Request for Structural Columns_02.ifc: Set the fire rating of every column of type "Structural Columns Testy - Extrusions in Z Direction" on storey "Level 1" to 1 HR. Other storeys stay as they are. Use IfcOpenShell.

First a look at what the model holds.

```python
import ifcopenshell
import ifcopenshell.util.element

model = ifcopenshell.open("Structural Columns_02.ifc")
print(model.schema)
storey = next(s for s in model.by_type("IfcBuildingStorey") if s.Name == "Level 1")
columns = [e for e in ifcopenshell.util.element.get_decomposition(storey) if e.is_a("IfcColumn")]
seen = {}
for e in columns:
    element_type = ifcopenshell.util.element.get_type(e)
    key = (element_type.Name if element_type != e and element_type else None, ifcopenshell.util.element.get_pset(e, "Pset_ColumnCommon", "FireRating"))
    seen[key] = seen.get(key, 0) + 1
for (name, value), count in sorted(seen.items(), key=str):
    print(count, "x", name, "|", value)
```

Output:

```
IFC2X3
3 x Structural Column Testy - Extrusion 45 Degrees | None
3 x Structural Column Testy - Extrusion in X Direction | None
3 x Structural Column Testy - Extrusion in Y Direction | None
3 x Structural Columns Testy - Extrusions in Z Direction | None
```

```python
import ifcopenshell
import ifcopenshell.api.pset
import ifcopenshell.util.element

model = ifcopenshell.open("Structural Columns_02.ifc")

storey = next(s for s in model.by_type("IfcBuildingStorey") if s.Name == "Level 1")
columns = [e for e in ifcopenshell.util.element.get_decomposition(storey) if e.is_a("IfcColumn")]

count = 0
for e in columns:
    element_type = ifcopenshell.util.element.get_type(e)
    if element_type in (None, e) or element_type.Name != "Structural Columns Testy - Extrusions in Z Direction":
        continue
    # add_pset returns the element's existing set when there is one.
    pset = ifcopenshell.api.pset.add_pset(model, product=e, name="Pset_ColumnCommon")
    ifcopenshell.api.pset.edit_pset(model, pset=pset, properties={"FireRating": "1 HR"})
    count += 1

print(count, "columns updated")

model.write("Structural Columns_02_edited.ifc")
```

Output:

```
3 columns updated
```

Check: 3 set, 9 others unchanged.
